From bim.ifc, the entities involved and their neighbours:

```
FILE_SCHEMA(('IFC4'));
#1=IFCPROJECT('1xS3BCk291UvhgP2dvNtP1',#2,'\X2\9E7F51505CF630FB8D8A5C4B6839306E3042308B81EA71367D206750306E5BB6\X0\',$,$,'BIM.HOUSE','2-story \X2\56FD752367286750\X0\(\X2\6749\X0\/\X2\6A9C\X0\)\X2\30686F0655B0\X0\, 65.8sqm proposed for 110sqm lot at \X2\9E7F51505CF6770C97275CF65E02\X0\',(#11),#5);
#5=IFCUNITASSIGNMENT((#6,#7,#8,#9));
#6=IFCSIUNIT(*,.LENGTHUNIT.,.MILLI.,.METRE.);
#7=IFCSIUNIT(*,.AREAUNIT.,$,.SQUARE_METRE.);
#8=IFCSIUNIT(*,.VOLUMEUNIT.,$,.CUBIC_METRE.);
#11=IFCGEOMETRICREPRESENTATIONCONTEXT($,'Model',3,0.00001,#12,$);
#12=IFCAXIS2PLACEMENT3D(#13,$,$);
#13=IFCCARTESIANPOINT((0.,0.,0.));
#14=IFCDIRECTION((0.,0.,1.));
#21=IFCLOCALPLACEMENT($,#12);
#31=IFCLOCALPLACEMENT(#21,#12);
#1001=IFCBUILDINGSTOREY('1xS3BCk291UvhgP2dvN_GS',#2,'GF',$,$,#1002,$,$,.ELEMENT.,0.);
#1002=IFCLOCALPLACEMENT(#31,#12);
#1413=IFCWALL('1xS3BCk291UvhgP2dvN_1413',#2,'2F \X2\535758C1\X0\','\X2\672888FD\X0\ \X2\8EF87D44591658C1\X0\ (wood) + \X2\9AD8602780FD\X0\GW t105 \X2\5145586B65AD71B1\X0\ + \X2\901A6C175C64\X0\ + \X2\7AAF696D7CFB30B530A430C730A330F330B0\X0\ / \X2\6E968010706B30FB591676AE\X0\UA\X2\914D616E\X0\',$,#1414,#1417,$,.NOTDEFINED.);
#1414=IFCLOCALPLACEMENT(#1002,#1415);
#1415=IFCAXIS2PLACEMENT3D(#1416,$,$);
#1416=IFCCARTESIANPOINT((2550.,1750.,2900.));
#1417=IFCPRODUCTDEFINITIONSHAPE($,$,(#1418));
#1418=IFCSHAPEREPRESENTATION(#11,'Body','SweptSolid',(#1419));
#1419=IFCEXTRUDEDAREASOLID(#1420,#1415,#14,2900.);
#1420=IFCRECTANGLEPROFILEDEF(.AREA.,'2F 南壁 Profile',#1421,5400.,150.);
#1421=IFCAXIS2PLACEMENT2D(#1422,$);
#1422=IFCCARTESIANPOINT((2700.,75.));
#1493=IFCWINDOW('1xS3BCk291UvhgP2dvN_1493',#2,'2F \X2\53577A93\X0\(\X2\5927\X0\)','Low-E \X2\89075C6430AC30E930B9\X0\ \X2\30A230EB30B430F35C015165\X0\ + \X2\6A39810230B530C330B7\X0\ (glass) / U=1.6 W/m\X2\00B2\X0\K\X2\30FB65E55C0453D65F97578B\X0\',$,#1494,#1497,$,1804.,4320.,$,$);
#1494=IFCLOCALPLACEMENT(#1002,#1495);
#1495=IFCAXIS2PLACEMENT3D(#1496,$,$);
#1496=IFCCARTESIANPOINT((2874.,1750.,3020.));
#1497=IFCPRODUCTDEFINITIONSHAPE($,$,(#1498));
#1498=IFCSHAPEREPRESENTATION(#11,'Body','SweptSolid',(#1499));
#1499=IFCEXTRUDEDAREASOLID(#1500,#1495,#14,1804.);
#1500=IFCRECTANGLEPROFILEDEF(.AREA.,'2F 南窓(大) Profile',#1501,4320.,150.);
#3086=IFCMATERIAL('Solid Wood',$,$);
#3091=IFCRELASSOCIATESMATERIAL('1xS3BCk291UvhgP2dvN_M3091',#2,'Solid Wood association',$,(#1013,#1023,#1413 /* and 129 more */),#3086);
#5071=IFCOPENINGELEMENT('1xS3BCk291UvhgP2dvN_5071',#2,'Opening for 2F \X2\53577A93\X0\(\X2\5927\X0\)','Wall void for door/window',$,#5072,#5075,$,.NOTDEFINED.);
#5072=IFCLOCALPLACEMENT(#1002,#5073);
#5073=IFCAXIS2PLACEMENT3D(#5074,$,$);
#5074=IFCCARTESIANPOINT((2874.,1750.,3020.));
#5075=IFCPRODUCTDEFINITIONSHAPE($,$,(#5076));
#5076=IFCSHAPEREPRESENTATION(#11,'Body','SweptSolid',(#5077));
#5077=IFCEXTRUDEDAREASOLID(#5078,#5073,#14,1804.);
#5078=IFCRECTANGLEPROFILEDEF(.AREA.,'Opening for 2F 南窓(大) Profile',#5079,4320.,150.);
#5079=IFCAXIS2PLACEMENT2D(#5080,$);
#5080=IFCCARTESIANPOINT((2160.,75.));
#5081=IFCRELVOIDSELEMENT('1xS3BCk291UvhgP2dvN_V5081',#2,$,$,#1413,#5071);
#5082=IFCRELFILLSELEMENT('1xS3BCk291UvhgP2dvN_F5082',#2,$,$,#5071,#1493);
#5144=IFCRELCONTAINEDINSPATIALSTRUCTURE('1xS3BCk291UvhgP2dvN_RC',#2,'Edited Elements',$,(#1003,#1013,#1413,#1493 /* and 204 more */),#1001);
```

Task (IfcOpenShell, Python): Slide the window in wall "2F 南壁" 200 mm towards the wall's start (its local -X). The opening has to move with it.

```python
import ifcopenshell
import ifcopenshell.api.geometry
import ifcopenshell.util.placement
import ifcopenshell.util.unit

model = ifcopenshell.open("bim.ifc")
unit_scale = ifcopenshell.util.unit.calculate_unit_scale(model)

window = model.by_guid("1xS3BCk291UvhgP2dvN_1493")
opening = window.FillsVoids[0].RelatingOpeningElement
wall = opening.VoidsElements[0].RelatingBuildingElement

wall_matrix = ifcopenshell.util.placement.get_local_placement(wall.ObjectPlacement)
shift = wall_matrix[:3, 0] * -0.2 / unit_scale
before = ifcopenshell.util.placement.get_local_placement(window.ObjectPlacement)[:3, 3].copy()

# The window is not placed relative to its opening, so move both.
for product in (opening, window):
    matrix = ifcopenshell.util.placement.get_local_placement(product.ObjectPlacement)
    matrix[:3, 3] += shift
    ifcopenshell.api.geometry.edit_object_placement(model, product=product, matrix=matrix, is_si=False)

after = ifcopenshell.util.placement.get_local_placement(window.ObjectPlacement)[:3, 3]
print("window moved by", (after - before).round(3) + 0.0)

model.write("bim_updated.ifc")
```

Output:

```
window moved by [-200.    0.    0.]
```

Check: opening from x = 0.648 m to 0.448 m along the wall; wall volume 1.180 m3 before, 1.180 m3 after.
